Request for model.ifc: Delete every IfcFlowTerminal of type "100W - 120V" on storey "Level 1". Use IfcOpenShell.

First a look at what the model holds.

```python
import ifcopenshell
import ifcopenshell.util.element

model = ifcopenshell.open("model.ifc")
print(model.schema)
storey = next(s for s in model.by_type("IfcBuildingStorey") if s.Name == "Level 1")
terminals = [e for e in ifcopenshell.util.element.get_decomposition(storey) if e.is_a("IfcFlowTerminal")]
seen = {}
for e in terminals:
    element_type = ifcopenshell.util.element.get_type(e)
    name = element_type.Name if element_type not in (None, e) else None
    seen[name] = seen.get(name, 0) + 1
for name, count in sorted(seen.items(), key=str):
    print(count, "x", name)
```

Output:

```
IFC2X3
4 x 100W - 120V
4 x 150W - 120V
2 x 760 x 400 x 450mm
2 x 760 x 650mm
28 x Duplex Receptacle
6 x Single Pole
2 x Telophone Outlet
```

```python
import ifcopenshell
import ifcopenshell.api.root
import ifcopenshell.util.element

model = ifcopenshell.open("model.ifc")

storey = next(s for s in model.by_type("IfcBuildingStorey") if s.Name == "Level 1")
terminals = [e for e in ifcopenshell.util.element.get_decomposition(storey) if e.is_a("IfcFlowTerminal")]
targets = [e for e in terminals if (t := ifcopenshell.util.element.get_type(e)) not in (None, e) and t.Name == "100W - 120V"]

for e in targets:
    ifcopenshell.api.root.remove_product(model, product=e)
print(len(targets), "removed")

model.write("model_updated.ifc")
```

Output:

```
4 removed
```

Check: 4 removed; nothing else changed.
